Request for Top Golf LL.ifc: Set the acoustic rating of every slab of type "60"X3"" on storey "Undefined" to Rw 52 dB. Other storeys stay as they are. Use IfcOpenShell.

First a look at what the model holds.

```python
import ifcopenshell
import ifcopenshell.util.element

model = ifcopenshell.open("Top Golf LL.ifc")
print(model.schema)
storey = next(s for s in model.by_type("IfcBuildingStorey") if s.Name == "Undefined")
slabs = [e for e in ifcopenshell.util.element.get_decomposition(storey) if e.is_a("IfcSlab")]
seen = {}
for e in slabs:
    element_type = ifcopenshell.util.element.get_type(e)
    key = (element_type.Name if element_type != e and element_type else None, ifcopenshell.util.element.get_pset(e, "Pset_SlabCommon", "AcousticRating"))
    seen[key] = seen.get(key, 0) + 1
for (name, value), count in sorted(seen.items(), key=str):
    print(count, "x", name, "|", value)
```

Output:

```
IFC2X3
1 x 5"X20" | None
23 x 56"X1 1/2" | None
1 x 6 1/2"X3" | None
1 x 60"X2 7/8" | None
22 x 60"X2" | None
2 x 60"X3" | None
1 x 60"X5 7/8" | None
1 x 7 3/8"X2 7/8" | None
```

```python
import ifcopenshell
import ifcopenshell.api.pset
import ifcopenshell.util.element

model = ifcopenshell.open("Top Golf LL.ifc")

storey = next(s for s in model.by_type("IfcBuildingStorey") if s.Name == "Undefined")
slabs = [e for e in ifcopenshell.util.element.get_decomposition(storey) if e.is_a("IfcSlab")]

count = 0
for e in slabs:
    element_type = ifcopenshell.util.element.get_type(e)
    if element_type in (None, e) or element_type.Name != '60"X3"':
        continue
    # add_pset returns the element's existing set when there is one.
    pset = ifcopenshell.api.pset.add_pset(model, product=e, name="Pset_SlabCommon")
    ifcopenshell.api.pset.edit_pset(model, pset=pset, properties={"AcousticRating": "Rw 52 dB"})
    count += 1

print(count, "slabs updated")

model.write("Top Golf LL_updated.ifc")
```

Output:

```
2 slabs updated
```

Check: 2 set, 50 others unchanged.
